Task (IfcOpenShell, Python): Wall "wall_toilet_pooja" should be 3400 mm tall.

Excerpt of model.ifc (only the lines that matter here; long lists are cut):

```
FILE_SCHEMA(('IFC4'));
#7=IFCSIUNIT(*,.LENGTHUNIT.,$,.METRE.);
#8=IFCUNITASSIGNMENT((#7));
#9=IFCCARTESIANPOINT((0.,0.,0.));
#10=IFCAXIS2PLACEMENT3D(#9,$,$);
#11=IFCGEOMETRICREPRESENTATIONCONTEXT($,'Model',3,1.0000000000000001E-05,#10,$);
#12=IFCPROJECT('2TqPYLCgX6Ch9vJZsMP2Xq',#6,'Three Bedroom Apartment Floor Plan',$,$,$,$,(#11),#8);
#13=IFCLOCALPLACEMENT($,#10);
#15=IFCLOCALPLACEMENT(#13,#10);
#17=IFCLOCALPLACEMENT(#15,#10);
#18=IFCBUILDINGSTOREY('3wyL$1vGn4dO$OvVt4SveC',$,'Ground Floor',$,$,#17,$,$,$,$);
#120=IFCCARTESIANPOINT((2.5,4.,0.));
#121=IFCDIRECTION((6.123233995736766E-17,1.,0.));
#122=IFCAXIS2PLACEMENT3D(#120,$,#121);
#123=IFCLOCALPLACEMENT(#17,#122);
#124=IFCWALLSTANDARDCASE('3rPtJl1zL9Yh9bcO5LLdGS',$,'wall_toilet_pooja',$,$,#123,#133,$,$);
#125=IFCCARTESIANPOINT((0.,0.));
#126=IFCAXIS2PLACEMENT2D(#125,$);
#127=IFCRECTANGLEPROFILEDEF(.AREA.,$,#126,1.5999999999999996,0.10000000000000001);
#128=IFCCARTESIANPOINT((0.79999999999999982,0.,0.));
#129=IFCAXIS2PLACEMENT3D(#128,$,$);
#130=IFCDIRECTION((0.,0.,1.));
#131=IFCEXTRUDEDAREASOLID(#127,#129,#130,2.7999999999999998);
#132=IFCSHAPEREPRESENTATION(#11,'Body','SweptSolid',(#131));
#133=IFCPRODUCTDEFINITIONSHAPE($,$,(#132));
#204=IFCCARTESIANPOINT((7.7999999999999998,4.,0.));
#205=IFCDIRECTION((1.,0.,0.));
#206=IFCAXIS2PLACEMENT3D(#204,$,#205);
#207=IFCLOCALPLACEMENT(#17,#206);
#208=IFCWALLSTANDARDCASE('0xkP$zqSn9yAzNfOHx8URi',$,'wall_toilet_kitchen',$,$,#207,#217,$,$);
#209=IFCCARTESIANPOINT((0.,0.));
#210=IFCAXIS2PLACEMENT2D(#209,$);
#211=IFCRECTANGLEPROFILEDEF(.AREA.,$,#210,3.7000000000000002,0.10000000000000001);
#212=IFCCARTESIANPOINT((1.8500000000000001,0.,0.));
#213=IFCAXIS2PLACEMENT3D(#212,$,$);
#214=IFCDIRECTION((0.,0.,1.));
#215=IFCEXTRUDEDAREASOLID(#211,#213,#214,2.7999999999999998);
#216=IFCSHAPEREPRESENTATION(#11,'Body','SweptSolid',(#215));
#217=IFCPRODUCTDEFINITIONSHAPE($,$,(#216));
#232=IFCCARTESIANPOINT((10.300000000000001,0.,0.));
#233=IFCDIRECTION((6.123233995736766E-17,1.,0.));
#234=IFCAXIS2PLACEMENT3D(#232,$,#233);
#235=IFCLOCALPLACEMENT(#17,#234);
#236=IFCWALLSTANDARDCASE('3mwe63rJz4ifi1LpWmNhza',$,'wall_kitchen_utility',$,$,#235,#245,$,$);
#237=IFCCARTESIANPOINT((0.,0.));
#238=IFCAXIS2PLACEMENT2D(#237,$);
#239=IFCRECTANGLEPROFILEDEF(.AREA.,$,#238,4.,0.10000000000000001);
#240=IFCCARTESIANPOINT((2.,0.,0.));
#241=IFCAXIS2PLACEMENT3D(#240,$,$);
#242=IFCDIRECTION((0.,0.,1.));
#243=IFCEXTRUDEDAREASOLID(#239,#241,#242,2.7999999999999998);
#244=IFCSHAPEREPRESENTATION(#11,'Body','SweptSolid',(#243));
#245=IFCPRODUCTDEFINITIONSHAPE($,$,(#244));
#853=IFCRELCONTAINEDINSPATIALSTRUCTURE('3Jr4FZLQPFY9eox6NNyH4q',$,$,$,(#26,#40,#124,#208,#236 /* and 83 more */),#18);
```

```python
import ifcopenshell
import ifcopenshell.geom
import ifcopenshell.util.shape
import ifcopenshell.util.unit

model = ifcopenshell.open("model.ifc")
unit_scale = ifcopenshell.util.unit.calculate_unit_scale(model)
settings = ifcopenshell.geom.settings()


def volume(element):
    """Net volume in cubic metres, openings subtracted."""
    shape = ifcopenshell.geom.create_shape(settings, element)
    return ifcopenshell.util.shape.get_volume(shape.geometry)


wall = model.by_guid("3rPtJl1zL9Yh9bcO5LLdGS")
before = volume(wall)

body = next(r for r in wall.Representation.Representations if r.RepresentationIdentifier == "Body")
solid = body.Items[0]
old_height = solid.Depth
solid.Depth = 3.4 / unit_scale
after = volume(wall)

print(f"height {old_height:g} -> {solid.Depth:g}, volume {before:.3f} -> {after:.3f} m3")

model.write("model_rev.ifc")
```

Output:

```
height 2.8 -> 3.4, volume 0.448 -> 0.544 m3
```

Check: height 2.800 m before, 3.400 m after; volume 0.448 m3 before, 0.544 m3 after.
